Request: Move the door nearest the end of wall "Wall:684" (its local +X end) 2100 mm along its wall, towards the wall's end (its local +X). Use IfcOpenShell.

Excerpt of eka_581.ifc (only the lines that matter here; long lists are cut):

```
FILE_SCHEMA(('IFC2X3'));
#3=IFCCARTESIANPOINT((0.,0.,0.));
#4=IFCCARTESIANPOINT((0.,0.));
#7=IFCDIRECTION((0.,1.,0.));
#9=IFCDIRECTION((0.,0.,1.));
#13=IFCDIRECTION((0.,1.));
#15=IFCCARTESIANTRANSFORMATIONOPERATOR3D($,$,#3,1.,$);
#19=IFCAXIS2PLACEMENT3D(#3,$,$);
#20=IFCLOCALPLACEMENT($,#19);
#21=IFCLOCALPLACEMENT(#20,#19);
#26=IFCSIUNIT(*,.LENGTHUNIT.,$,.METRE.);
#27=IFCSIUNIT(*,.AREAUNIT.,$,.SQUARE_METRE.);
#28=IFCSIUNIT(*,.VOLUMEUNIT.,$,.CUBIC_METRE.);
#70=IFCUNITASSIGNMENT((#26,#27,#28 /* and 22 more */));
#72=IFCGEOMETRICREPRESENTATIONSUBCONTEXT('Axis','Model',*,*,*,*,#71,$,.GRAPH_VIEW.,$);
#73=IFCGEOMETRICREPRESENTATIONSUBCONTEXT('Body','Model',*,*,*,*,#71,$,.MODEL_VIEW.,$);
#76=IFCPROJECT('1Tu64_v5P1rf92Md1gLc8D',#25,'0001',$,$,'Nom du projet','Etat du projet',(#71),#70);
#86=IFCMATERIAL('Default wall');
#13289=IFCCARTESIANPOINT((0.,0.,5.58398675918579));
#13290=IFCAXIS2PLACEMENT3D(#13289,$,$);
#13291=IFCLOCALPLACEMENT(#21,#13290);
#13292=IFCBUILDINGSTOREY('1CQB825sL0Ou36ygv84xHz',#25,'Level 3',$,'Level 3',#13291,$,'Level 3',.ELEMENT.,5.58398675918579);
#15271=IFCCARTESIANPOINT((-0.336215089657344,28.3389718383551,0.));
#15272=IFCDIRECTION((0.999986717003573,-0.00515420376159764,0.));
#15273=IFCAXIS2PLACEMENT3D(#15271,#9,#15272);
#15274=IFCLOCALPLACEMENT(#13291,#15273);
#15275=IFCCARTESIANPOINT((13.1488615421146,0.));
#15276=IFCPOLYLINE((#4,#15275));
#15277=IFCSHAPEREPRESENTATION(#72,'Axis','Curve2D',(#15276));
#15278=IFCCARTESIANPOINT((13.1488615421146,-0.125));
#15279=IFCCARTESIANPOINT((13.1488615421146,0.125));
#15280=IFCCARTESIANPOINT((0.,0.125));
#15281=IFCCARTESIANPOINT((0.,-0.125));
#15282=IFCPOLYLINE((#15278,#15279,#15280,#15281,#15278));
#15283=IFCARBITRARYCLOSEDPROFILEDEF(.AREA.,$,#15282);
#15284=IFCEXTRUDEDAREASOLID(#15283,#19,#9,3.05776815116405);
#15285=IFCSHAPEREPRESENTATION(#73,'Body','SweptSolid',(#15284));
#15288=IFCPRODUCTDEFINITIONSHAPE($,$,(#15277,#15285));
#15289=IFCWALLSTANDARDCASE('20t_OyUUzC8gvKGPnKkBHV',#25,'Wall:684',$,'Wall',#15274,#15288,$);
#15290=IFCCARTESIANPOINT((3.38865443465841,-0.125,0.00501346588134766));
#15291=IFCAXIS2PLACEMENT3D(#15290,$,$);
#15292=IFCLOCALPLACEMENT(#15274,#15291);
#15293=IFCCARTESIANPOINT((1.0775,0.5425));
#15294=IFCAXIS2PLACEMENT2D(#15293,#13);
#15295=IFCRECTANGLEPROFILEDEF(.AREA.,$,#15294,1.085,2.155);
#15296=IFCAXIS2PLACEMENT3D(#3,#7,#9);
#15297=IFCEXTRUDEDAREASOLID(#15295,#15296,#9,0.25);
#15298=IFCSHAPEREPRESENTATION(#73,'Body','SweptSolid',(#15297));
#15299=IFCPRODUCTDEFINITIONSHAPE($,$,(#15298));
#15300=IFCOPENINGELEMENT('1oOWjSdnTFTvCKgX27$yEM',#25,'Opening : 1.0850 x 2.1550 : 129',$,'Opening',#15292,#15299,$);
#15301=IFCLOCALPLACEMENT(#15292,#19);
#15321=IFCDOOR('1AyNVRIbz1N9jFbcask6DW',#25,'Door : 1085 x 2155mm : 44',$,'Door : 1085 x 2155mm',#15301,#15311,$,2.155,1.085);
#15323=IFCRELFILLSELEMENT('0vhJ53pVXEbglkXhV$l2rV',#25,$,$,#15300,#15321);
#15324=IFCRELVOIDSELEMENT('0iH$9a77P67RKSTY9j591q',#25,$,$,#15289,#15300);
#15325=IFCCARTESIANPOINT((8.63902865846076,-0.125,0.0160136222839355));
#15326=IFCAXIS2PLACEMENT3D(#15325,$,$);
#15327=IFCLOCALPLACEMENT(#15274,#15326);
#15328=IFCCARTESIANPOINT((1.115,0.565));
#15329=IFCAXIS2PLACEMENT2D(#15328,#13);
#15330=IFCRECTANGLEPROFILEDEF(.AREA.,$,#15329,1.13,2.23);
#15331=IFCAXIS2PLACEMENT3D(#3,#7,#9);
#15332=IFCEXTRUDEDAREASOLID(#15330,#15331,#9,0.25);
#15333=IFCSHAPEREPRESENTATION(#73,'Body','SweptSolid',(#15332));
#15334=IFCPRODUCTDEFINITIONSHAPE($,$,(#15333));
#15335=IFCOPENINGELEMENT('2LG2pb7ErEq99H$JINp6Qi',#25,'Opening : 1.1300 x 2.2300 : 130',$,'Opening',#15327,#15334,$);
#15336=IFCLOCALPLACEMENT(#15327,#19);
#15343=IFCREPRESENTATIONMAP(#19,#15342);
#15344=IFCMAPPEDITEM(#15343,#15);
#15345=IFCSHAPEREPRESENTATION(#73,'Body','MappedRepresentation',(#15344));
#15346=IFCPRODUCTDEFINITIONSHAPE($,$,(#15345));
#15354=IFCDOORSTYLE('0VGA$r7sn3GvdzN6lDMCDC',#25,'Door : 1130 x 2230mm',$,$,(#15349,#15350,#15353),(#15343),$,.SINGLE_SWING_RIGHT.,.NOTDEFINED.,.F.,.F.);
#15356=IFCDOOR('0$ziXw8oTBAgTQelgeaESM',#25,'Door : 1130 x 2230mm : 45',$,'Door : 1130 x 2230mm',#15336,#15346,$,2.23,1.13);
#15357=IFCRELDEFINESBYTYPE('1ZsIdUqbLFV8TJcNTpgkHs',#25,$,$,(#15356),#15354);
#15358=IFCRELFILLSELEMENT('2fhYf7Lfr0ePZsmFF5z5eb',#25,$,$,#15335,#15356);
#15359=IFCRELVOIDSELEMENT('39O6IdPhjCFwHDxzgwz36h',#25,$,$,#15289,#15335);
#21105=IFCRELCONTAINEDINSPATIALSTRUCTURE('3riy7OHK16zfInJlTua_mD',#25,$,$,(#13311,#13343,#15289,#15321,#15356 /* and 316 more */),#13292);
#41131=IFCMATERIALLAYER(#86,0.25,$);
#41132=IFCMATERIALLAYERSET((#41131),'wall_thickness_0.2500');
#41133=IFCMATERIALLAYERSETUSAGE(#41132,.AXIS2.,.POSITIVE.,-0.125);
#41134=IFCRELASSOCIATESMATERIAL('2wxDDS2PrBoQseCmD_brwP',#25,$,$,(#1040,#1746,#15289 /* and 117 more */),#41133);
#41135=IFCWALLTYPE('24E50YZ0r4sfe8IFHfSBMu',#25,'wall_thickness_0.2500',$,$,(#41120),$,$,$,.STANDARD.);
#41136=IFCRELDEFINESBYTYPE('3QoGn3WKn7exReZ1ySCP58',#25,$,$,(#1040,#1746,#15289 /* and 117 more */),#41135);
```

```python
import ifcopenshell
import ifcopenshell.api.geometry
import ifcopenshell.util.placement
import ifcopenshell.util.unit

model = ifcopenshell.open("eka_581.ifc")
unit_scale = ifcopenshell.util.unit.calculate_unit_scale(model)

door = model.by_guid("0$ziXw8oTBAgTQelgeaESM")
opening = door.FillsVoids[0].RelatingOpeningElement
wall = opening.VoidsElements[0].RelatingBuildingElement

wall_matrix = ifcopenshell.util.placement.get_local_placement(wall.ObjectPlacement)
shift = wall_matrix[:3, 0] * 2.1 / unit_scale
before = ifcopenshell.util.placement.get_local_placement(door.ObjectPlacement)[:3, 3].copy()

# The door is placed relative to its opening, so it follows when the opening moves.
matrix = ifcopenshell.util.placement.get_local_placement(opening.ObjectPlacement)
matrix[:3, 3] += shift
ifcopenshell.api.geometry.edit_object_placement(
    model, product=opening, matrix=matrix, is_si=False, should_transform_children=True
)

after = ifcopenshell.util.placement.get_local_placement(door.ObjectPlacement)[:3, 3]
print("door moved by", (after - before).round(3) + 0.0)

model.write("eka_581_rev.ifc")
```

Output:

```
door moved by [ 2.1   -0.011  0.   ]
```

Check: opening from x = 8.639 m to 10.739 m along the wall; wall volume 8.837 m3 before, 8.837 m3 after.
